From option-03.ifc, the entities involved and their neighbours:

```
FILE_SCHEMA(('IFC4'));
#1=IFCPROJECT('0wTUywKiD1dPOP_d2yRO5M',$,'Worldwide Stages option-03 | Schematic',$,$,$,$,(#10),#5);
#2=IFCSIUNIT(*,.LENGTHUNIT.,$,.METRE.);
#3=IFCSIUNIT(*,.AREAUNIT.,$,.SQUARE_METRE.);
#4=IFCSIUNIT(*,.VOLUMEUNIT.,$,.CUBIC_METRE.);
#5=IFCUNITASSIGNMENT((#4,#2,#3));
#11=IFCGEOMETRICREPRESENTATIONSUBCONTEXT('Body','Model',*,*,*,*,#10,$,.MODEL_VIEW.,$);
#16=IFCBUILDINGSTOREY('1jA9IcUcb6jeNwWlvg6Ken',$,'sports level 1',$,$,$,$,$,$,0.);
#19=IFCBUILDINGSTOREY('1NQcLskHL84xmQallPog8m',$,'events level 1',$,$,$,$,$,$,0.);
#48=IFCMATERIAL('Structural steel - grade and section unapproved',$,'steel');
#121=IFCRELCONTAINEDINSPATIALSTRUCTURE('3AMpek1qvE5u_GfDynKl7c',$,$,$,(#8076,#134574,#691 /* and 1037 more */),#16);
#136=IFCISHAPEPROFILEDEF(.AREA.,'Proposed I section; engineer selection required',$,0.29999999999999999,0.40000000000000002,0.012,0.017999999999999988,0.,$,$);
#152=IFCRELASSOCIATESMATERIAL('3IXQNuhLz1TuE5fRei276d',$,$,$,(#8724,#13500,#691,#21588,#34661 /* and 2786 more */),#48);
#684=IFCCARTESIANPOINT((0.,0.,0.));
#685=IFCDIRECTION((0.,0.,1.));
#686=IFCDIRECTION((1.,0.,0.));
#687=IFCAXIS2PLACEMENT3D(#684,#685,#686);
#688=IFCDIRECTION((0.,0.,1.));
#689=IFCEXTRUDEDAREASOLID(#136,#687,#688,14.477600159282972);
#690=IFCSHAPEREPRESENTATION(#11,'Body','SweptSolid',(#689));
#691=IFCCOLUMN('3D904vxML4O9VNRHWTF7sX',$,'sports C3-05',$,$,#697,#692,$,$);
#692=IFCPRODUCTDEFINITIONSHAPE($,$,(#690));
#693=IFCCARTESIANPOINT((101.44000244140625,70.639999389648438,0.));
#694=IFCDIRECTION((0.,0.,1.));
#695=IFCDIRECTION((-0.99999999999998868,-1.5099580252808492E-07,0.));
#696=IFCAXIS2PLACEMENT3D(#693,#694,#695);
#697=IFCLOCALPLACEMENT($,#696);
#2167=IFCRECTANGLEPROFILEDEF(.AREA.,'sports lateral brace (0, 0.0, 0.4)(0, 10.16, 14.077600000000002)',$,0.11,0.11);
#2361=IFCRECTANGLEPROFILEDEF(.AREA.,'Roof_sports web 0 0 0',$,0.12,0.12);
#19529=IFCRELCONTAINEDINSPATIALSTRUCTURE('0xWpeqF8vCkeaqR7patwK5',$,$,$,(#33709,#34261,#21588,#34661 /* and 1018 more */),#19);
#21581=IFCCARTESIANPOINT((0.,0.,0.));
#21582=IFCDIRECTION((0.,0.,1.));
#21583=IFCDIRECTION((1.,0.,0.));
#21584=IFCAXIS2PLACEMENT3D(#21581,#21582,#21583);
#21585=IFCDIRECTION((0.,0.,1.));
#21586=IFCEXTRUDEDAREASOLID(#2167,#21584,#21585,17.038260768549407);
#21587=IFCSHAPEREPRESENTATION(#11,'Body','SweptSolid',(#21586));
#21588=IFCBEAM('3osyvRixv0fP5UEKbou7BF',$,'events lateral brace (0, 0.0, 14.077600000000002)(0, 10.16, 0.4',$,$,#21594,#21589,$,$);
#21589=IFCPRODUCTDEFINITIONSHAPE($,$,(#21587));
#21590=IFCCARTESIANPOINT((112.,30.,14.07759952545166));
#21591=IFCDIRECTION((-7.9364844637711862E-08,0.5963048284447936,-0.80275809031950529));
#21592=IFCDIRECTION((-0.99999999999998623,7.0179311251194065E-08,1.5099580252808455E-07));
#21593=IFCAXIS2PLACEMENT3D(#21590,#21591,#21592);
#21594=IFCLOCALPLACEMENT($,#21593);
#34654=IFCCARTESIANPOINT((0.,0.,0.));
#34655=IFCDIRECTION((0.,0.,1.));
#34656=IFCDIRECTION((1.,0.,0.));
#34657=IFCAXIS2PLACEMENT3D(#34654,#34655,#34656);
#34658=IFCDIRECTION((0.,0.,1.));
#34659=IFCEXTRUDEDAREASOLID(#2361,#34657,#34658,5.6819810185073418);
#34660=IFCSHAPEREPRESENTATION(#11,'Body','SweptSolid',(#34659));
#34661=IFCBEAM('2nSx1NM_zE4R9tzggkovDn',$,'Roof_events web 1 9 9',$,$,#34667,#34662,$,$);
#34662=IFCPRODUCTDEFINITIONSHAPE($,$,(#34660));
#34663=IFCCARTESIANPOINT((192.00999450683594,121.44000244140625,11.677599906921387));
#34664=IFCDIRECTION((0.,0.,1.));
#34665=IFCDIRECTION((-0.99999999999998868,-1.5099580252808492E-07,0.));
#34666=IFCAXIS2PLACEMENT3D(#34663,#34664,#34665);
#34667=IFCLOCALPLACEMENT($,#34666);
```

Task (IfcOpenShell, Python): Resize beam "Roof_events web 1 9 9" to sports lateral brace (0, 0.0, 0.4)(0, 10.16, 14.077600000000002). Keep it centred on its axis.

```python
import ifcopenshell
import ifcopenshell.util.element
import ifcopenshell.util.representation

model = ifcopenshell.open("option-03.ifc")

member = model.by_guid("2nSx1NM_zE4R9tzggkovDn")
source = next(p for p in model.by_type("IfcRectangleProfileDef") if p.ProfileName == "sports lateral brace (0, 0.0, 0.4)(0, 10.16, 14.077600000000002)")

body = ifcopenshell.util.representation.get_representation(member, "Model", "Body")
solid = body.Items[0]
old_profile = solid.SweptArea

# Copy the section's sizes but keep this member's own profile position.
profile = ifcopenshell.util.element.copy(model, source)
profile.Position = old_profile.Position
solid.SweptArea = profile
if not model.get_total_inverses(old_profile):
    ifcopenshell.util.element.remove_deep2(model, old_profile)

print(solid.SweptArea)

model.write("option-03_rev.ifc")
```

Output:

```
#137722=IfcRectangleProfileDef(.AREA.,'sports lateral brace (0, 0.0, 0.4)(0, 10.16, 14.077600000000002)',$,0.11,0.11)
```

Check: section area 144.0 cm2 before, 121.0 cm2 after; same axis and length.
